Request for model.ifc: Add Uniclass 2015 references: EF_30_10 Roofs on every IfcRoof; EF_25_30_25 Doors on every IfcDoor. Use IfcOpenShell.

First a look at what the model holds.

```python
import ifcopenshell

model = ifcopenshell.open("model.ifc")
print(model.schema)
print("classifications:", [c.Name for c in model.by_type("IfcClassification")])
for ifc_class in ("IfcDoor", "IfcRoof", "IfcStair", "IfcWall", "IfcWindow"):
    print(ifc_class, len(model.by_type(ifc_class)))
```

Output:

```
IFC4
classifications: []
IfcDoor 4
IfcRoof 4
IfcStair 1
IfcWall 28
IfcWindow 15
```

```python
import ifcopenshell
import ifcopenshell.api.classification

model = ifcopenshell.open("model.ifc")

system = ifcopenshell.api.classification.add_classification(model, classification="Uniclass 2015")

codes = {
    "IfcRoof": ("EF_30_10", "Roofs"),
    "IfcDoor": ("EF_25_30_25", "Doors"),
}
for ifc_class, (code, name) in codes.items():
    products = model.by_type(ifc_class)
    ifcopenshell.api.classification.add_reference(
        model, products=products, classification=system, identification=code, name=name
    )
    print(code, len(products))

model.write("model_updated.ifc")
```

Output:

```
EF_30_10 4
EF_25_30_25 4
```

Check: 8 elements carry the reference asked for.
